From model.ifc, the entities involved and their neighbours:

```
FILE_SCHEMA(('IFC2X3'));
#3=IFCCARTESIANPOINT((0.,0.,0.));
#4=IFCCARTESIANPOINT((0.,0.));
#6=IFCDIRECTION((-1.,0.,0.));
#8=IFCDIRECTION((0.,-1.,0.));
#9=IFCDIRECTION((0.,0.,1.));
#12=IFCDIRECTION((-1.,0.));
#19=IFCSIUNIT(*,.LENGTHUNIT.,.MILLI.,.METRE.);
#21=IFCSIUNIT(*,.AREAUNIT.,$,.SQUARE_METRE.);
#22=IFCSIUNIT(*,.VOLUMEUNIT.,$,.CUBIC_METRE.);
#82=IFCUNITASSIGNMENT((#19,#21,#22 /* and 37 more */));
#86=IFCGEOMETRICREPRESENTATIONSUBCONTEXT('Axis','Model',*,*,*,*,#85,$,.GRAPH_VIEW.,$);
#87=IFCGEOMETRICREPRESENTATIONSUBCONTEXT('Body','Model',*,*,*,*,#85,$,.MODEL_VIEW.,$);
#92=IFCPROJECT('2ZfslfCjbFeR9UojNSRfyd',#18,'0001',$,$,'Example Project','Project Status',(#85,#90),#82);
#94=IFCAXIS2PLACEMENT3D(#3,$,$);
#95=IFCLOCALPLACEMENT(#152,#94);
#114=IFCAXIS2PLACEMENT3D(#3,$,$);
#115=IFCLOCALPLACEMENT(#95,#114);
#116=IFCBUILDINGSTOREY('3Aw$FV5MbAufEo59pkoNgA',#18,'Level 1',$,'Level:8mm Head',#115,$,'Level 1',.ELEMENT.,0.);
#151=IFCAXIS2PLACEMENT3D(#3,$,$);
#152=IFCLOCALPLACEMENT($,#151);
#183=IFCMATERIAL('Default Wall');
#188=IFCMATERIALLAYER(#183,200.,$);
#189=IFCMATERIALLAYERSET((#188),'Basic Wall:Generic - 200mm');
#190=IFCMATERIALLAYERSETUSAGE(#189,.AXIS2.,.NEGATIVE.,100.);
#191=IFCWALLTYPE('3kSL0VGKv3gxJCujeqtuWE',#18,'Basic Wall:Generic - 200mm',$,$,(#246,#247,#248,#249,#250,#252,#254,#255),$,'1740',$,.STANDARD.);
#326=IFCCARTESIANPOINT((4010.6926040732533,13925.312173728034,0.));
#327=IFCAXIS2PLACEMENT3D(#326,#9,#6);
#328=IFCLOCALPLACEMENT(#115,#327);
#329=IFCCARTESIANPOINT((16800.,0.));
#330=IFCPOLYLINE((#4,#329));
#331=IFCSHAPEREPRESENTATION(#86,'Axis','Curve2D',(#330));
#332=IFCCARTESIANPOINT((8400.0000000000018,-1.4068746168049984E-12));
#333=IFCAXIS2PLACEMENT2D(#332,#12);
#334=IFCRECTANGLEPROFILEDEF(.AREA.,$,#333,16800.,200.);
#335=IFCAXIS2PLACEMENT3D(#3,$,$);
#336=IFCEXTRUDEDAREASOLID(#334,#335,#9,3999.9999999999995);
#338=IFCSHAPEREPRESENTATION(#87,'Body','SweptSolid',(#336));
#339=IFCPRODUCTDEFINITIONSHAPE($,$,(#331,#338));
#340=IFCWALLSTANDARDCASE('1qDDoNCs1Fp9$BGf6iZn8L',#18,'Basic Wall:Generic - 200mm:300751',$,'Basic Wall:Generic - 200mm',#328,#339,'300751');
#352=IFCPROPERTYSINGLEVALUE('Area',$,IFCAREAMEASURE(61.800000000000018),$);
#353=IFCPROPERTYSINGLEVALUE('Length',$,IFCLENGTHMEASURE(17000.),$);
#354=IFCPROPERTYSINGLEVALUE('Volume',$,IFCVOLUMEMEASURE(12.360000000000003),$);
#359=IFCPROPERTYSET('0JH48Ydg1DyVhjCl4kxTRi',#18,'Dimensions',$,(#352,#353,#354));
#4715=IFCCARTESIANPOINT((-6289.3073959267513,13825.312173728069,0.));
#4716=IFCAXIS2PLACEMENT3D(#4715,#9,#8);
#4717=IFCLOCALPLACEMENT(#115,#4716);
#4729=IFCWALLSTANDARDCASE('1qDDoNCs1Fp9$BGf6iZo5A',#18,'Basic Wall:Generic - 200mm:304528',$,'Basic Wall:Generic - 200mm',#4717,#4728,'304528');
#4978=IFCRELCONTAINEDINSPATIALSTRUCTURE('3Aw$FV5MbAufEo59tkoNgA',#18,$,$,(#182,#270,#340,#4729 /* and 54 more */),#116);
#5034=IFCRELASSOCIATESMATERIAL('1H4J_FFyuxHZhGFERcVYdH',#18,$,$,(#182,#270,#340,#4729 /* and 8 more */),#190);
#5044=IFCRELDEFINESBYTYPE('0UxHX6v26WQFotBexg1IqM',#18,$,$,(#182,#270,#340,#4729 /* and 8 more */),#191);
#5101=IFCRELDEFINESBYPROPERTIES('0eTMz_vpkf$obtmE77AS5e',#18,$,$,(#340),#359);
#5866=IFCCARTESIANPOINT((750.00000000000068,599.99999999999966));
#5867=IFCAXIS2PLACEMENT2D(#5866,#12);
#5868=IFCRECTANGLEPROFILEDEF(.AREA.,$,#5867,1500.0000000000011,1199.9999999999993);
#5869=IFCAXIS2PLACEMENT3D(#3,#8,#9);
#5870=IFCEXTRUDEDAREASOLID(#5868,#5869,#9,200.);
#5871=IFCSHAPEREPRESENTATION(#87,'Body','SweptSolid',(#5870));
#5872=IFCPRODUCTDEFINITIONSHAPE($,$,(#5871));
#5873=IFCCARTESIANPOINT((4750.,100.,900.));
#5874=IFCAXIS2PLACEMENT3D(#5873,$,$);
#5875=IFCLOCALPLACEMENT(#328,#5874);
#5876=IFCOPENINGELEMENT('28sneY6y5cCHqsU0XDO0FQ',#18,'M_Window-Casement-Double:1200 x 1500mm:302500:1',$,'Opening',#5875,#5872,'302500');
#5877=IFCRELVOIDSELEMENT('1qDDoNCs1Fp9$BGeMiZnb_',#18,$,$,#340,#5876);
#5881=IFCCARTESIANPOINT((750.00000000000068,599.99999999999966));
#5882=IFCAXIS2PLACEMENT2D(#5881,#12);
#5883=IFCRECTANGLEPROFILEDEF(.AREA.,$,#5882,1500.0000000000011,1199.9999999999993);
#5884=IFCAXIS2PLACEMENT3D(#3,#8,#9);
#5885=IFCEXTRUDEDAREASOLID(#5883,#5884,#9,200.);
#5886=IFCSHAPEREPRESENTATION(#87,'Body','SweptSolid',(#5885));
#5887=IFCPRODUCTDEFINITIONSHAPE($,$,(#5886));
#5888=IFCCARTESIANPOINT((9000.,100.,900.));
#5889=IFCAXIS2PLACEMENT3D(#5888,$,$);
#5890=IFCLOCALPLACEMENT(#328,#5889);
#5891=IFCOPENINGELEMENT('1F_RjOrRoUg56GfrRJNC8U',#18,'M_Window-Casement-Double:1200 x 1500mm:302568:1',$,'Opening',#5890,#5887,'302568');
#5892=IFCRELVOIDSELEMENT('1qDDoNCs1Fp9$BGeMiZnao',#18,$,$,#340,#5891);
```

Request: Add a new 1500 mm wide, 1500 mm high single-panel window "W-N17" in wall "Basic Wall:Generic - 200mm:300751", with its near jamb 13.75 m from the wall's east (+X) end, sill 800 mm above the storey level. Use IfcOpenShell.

```python
import numpy as np
import ifcopenshell
import ifcopenshell.api.feature
import ifcopenshell.api.geometry
import ifcopenshell.api.pset
import ifcopenshell.api.root
import ifcopenshell.api.spatial
import ifcopenshell.api.type
import ifcopenshell.geom
import ifcopenshell.util.element
import ifcopenshell.util.placement
import ifcopenshell.util.representation
import ifcopenshell.util.shape
import ifcopenshell.util.unit

model = ifcopenshell.open("model.ifc")
unit_scale = ifcopenshell.util.unit.calculate_unit_scale(model)
area_scale = ifcopenshell.util.unit.calculate_unit_scale(model, "AREAUNIT")
volume_scale = ifcopenshell.util.unit.calculate_unit_scale(model, "VOLUMEUNIT")
settings = ifcopenshell.geom.settings()


def volume(element):
    """Net volume in cubic metres, openings subtracted."""
    shape = ifcopenshell.geom.create_shape(settings, element)
    return ifcopenshell.util.shape.get_volume(shape.geometry)


wall = model.by_guid("1qDDoNCs1Fp9$BGf6iZn8L")
storey = ifcopenshell.util.element.get_container(wall, ifc_class="IfcBuildingStorey")
context = ifcopenshell.util.representation.get_context(model, "Model", "Body", "MODEL_VIEW")
before = volume(wall)

width, height, from_end, sill = 1.5, 1.5, 13.75, 0.8  # metres

# The wall runs along its own X axis, and the end named is its -X end.
wall_shape = ifcopenshell.geom.create_shape(settings, wall)
x, y, z = ifcopenshell.util.shape.get_vertices(wall_shape.geometry).T
start = x.min() + from_end
face, thickness = float(y.min()), float(y.max() - y.min())
wall_matrix = ifcopenshell.util.placement.get_local_placement(wall.ObjectPlacement)
level = ifcopenshell.util.placement.get_local_placement(storey.ObjectPlacement)[2, 3]


def in_wall(x, y):
    """Placement at x, y metres in the wall's axes, at sill height."""
    matrix = wall_matrix.copy()
    matrix[:, 3] = wall_matrix @ np.array([x / unit_scale, y / unit_scale, 0.0, 1.0])
    matrix[2, 3] = level + sill / unit_scale
    return matrix


# Opening: a box that overshoots both wall faces by 50 mm.
opening = ifcopenshell.api.root.create_entity(model, ifc_class="IfcOpeningElement")
box = ifcopenshell.api.geometry.add_wall_representation(
    model, context=context, length=width, height=height, thickness=thickness + 0.1
)
ifcopenshell.api.geometry.assign_representation(model, product=opening, representation=box)
ifcopenshell.api.geometry.edit_object_placement(model, product=opening, matrix=in_wall(start, face - 0.05), is_si=False)
ifcopenshell.api.feature.add_feature(model, feature=opening, element=wall)

window = ifcopenshell.api.root.create_entity(model, ifc_class="IfcWindow", name="W-N17")
window.OverallWidth, window.OverallHeight = width / unit_scale, height / unit_scale
body = ifcopenshell.api.geometry.add_window_representation(
    model,
    context=context,
    overall_width=window.OverallWidth,
    overall_height=window.OverallHeight,
    partition_type="SINGLE_PANEL",
)
ifcopenshell.api.geometry.assign_representation(model, product=window, representation=body)
ifcopenshell.api.spatial.assign_container(model, products=[window], relating_structure=storey)
fills = ifcopenshell.api.feature.add_filling(model, opening=opening, element=window)
fills.OwnerHistory = window.OwnerHistory  # required in IFC2X3

# IFC2X3 keeps the operation on the window style.
style = ifcopenshell.api.root.create_entity(model, ifc_class="IfcWindowStyle", name="W-N17")
style.OperationType, style.ConstructionType = "SINGLE_PANEL", "NOTDEFINED"
style.ParameterTakesPrecedence = style.Sizeable = False
ifcopenshell.api.type.assign_type(model, related_objects=[window], relating_type=style)

# Centre the window in the wall's thickness.
ifcopenshell.api.geometry.edit_object_placement(model, product=window, matrix=in_wall(start, face), is_si=False)
window_shape = ifcopenshell.geom.create_shape(settings, window)
depth = ifcopenshell.util.shape.get_vertices(window_shape.geometry)[:, 1]
offset = face + thickness / 2 - (depth.min() + depth.max()) / 2
ifcopenshell.api.geometry.edit_object_placement(model, product=window, matrix=in_wall(start, offset), is_si=False)

after = volume(wall)

# Update the wall's stored quantities.
pset = model.by_id(ifcopenshell.util.element.get_pset(wall, "Dimensions", should_inherit=False)["id"])
ifcopenshell.api.pset.edit_pset(model, pset=pset, properties={
    "Area": model.create_entity("IfcAreaMeasure", after / thickness / area_scale),
    "Volume": model.create_entity("IfcVolumeMeasure", after / volume_scale),
})

print(f"wall volume {before:.3f} -> {after:.3f} m3")

model.write("model_edited.ifc")
```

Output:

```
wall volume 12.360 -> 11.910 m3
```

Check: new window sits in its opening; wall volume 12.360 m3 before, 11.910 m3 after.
